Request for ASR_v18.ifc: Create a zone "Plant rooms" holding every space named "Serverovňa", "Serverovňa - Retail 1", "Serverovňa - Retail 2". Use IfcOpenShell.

First a look at what the model holds.

```python
import ifcopenshell

model = ifcopenshell.open("ASR_v18.ifc")
print(model.schema)
seen = {}
for space in model.by_type("IfcSpace"):
    seen[space.LongName] = seen.get(space.LongName, 0) + 1
for name, count in sorted(seen.items(), key=str):
    print(count, "x", name)
print("zones:", [z.Name for z in model.by_type("IfcZone")][:20])
```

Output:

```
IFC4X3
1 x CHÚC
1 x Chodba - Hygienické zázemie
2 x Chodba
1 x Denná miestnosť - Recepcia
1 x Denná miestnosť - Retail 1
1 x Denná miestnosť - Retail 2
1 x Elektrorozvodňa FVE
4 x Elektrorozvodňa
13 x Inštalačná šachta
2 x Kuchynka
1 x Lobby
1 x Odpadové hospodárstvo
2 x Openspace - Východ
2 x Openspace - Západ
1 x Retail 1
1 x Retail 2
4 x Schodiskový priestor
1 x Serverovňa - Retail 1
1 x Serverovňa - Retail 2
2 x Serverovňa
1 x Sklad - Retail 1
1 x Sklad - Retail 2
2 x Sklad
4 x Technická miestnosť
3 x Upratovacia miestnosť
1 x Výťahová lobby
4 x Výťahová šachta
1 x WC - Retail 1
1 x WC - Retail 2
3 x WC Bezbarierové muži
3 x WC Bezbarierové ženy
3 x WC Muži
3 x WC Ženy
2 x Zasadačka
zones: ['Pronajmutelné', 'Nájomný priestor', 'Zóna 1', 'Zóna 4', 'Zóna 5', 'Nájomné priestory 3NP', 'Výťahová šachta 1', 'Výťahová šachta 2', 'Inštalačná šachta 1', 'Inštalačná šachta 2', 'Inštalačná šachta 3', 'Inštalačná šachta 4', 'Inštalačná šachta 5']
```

```python
import ifcopenshell
import ifcopenshell.api.group
import ifcopenshell.api.root

model = ifcopenshell.open("ASR_v18.ifc")

names = {"Serverovňa", "Serverovňa - Retail 1", "Serverovňa - Retail 2"}
spaces = [s for s in model.by_type("IfcSpace") if s.LongName in names]

zone = ifcopenshell.api.root.create_entity(model, ifc_class="IfcZone", name="Plant rooms")
ifcopenshell.api.group.assign_group(model, products=spaces, group=zone)
print(len(spaces), "spaces in", zone.Name)

model.write("ASR_v18-out.ifc")
```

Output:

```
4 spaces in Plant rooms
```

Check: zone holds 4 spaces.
